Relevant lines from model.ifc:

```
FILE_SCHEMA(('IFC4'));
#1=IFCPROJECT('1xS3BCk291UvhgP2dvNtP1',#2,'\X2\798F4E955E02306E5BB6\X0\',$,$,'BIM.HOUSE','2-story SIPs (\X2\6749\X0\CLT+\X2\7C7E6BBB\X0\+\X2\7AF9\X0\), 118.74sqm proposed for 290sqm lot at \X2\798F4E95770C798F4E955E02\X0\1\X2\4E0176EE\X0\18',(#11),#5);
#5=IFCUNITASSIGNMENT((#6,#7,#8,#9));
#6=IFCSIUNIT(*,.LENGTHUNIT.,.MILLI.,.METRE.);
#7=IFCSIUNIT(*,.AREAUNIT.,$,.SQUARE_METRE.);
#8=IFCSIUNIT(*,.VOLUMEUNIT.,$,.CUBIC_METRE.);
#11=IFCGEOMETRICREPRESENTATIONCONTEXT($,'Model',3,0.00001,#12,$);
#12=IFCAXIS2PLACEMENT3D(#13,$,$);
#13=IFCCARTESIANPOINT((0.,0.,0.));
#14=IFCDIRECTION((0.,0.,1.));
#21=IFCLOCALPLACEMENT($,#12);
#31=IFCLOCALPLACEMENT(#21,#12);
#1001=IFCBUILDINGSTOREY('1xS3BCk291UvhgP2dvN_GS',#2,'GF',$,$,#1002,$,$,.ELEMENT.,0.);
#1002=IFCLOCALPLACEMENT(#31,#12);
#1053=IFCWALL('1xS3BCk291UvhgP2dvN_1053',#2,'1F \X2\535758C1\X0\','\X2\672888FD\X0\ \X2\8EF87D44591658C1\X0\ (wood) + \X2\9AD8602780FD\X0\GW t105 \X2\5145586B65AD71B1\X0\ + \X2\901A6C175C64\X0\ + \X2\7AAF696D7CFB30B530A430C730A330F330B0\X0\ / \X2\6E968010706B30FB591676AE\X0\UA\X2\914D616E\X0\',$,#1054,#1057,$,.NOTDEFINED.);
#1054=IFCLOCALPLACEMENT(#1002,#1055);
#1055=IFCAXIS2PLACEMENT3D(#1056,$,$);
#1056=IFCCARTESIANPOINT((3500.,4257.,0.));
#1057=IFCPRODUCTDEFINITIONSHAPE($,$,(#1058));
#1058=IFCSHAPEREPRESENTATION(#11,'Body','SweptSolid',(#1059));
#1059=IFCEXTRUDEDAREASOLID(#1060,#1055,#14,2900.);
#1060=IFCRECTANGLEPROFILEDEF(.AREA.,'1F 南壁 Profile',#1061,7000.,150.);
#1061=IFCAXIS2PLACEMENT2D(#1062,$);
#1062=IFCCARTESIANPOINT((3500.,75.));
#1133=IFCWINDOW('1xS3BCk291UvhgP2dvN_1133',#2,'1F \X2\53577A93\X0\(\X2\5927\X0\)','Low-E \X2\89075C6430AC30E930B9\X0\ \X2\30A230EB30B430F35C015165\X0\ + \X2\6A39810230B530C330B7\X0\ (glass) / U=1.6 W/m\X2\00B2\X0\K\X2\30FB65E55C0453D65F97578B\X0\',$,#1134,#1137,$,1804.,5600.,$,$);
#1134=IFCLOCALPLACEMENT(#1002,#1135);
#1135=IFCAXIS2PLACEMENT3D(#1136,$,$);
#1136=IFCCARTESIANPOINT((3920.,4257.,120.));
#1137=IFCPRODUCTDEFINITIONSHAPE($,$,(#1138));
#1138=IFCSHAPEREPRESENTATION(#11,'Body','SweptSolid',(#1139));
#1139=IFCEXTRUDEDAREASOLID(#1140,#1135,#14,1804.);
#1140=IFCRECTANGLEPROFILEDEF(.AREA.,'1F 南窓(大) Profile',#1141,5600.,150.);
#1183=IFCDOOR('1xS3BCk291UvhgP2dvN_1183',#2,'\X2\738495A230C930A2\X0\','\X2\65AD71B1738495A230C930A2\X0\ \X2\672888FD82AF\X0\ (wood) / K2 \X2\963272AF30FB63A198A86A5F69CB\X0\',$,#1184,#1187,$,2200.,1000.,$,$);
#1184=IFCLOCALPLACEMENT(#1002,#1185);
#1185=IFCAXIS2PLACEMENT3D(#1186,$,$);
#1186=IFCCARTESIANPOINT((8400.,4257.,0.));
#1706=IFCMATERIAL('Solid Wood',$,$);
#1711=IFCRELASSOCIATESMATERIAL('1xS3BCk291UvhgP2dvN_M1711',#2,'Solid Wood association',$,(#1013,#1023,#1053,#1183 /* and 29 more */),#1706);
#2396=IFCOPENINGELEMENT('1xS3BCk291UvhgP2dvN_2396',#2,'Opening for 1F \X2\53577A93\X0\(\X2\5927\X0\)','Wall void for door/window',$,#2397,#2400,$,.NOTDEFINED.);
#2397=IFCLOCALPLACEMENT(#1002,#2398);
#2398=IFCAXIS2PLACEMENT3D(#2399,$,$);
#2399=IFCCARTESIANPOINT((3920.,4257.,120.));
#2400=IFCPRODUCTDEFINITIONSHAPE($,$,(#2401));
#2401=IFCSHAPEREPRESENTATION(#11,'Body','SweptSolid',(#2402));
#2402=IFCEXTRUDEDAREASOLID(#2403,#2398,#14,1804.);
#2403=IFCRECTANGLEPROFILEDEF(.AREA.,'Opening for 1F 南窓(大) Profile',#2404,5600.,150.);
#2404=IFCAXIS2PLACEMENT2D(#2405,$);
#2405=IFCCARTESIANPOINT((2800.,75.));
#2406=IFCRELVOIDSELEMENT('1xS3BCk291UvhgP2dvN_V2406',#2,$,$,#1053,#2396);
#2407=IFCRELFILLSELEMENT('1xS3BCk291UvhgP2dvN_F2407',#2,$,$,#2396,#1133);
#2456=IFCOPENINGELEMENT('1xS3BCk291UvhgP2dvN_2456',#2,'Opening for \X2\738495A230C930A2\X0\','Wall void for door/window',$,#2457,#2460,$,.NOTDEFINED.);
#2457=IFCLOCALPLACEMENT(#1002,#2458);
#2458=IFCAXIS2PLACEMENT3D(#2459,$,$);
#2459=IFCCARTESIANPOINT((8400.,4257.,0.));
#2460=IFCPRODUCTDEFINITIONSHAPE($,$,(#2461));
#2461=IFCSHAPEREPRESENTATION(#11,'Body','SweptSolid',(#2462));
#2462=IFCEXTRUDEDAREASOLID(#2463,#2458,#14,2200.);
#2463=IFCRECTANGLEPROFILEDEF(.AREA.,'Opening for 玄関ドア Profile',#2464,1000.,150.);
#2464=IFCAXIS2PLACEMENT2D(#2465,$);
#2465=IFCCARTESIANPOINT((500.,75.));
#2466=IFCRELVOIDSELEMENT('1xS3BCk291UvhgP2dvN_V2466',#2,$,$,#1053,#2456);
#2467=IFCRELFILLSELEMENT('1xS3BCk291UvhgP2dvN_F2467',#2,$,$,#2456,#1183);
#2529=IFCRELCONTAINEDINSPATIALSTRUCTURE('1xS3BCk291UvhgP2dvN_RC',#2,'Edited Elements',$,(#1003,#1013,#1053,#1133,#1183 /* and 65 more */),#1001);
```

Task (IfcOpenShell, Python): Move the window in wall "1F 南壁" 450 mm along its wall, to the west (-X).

```python
import ifcopenshell
import ifcopenshell.api.geometry
import ifcopenshell.util.placement

model = ifcopenshell.open("model.ifc")

window = model.by_id(1133)
opening = window.FillsVoids[0].RelatingOpeningElement
wall = opening.VoidsElements[0].RelatingBuildingElement

wall_matrix = ifcopenshell.util.placement.get_local_placement(wall.ObjectPlacement)
shift = wall_matrix[:3, 0] * -450.0
before = ifcopenshell.util.placement.get_local_placement(window.ObjectPlacement)[:3, 3].copy()

# The window is not placed relative to its opening, so move both.
for product in (opening, window):
    matrix = ifcopenshell.util.placement.get_local_placement(product.ObjectPlacement)
    matrix[:3, 3] += shift
    ifcopenshell.api.geometry.edit_object_placement(model, product=product, matrix=matrix, is_si=False)

after = ifcopenshell.util.placement.get_local_placement(window.ObjectPlacement)[:3, 3]
print("window moved by", (after - before).round(3) + 0.0)

model.write("model-out.ifc")
```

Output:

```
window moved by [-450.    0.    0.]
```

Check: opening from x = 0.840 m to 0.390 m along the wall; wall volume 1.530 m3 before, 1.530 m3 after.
